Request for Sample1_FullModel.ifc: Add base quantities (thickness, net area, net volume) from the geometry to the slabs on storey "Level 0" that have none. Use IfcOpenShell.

First a look at what the model holds.

```python
import ifcopenshell
import ifcopenshell.util.element
import ifcopenshell.util.unit

model = ifcopenshell.open("Sample1_FullModel.ifc")
print(model.schema)
for unit_type in ("LENGTHUNIT", "AREAUNIT", "VOLUMEUNIT"):
    print(unit_type, ifcopenshell.util.unit.calculate_unit_scale(model, unit_type))
storey = next(s for s in model.by_type("IfcBuildingStorey") if s.Name == "Level 0")
slabs = [e for e in ifcopenshell.util.element.get_decomposition(storey) if e.is_a("IfcSlab")]
for e in sorted(slabs, key=lambda e: e.id()):
    print(e.id(), e.is_a(), e.Name, list(ifcopenshell.util.element.get_psets(e, qtos_only=True)), sep=" | ")
```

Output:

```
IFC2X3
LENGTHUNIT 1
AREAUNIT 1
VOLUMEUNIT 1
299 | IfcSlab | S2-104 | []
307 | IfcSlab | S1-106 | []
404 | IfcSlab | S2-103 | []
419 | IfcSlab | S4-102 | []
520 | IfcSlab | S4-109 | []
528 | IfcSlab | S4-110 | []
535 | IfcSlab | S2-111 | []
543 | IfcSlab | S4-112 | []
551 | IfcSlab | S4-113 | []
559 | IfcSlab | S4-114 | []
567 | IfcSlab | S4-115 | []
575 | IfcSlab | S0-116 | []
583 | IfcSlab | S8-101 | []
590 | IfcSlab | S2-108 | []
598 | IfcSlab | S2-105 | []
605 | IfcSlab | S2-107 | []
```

```python
import ifcopenshell
import ifcopenshell.api.pset
import ifcopenshell.geom
import ifcopenshell.util.element
import ifcopenshell.util.shape
import ifcopenshell.util.unit

model = ifcopenshell.open("Sample1_FullModel.ifc")
unit_scale = ifcopenshell.util.unit.calculate_unit_scale(model)
area_scale = ifcopenshell.util.unit.calculate_unit_scale(model, "AREAUNIT")
volume_scale = ifcopenshell.util.unit.calculate_unit_scale(model, "VOLUMEUNIT")
settings = ifcopenshell.geom.settings()

storey = next(s for s in model.by_type("IfcBuildingStorey") if s.Name == "Level 0")
slabs = [e for e in ifcopenshell.util.element.get_decomposition(storey) if e.is_a("IfcSlab")]

for e in sorted(slabs, key=lambda e: e.id()):
    if ifcopenshell.util.element.get_psets(e, qtos_only=True, should_inherit=False):
        continue
    # Geometry comes back in metres, in the element's own axes.
    shape = ifcopenshell.geom.create_shape(settings, e)
    values = {
        "Width": ifcopenshell.util.shape.get_z(shape.geometry) / unit_scale,
        "NetArea": ifcopenshell.util.shape.get_footprint_area(shape.geometry) / area_scale,
        "NetVolume": ifcopenshell.util.shape.get_volume(shape.geometry) / volume_scale,
    }
    qto = ifcopenshell.api.pset.add_qto(model, product=e, name="BaseQuantities")
    ifcopenshell.api.pset.edit_qto(model, qto=qto, properties=values)
    print(e.id(), {k: round(v, 3) for k, v in values.items()})

model.write("Sample1_FullModel_edited.ifc")
```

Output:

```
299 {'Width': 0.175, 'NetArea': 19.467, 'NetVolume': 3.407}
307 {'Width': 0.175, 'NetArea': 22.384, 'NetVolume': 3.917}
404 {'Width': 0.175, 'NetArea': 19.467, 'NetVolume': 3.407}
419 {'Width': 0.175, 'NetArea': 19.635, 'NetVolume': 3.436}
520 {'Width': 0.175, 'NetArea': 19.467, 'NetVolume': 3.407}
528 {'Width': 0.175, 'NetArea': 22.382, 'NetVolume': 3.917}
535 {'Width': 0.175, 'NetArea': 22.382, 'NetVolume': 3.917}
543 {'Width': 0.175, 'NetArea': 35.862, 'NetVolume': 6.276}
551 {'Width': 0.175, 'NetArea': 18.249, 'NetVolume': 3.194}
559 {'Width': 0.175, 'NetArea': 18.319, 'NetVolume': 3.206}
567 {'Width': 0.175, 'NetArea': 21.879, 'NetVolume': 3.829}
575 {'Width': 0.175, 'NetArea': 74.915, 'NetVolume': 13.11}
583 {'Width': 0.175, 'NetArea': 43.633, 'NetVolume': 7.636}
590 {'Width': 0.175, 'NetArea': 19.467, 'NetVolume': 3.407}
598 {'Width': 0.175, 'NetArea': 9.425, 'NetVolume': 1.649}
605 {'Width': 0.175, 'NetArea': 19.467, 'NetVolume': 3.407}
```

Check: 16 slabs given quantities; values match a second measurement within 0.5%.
